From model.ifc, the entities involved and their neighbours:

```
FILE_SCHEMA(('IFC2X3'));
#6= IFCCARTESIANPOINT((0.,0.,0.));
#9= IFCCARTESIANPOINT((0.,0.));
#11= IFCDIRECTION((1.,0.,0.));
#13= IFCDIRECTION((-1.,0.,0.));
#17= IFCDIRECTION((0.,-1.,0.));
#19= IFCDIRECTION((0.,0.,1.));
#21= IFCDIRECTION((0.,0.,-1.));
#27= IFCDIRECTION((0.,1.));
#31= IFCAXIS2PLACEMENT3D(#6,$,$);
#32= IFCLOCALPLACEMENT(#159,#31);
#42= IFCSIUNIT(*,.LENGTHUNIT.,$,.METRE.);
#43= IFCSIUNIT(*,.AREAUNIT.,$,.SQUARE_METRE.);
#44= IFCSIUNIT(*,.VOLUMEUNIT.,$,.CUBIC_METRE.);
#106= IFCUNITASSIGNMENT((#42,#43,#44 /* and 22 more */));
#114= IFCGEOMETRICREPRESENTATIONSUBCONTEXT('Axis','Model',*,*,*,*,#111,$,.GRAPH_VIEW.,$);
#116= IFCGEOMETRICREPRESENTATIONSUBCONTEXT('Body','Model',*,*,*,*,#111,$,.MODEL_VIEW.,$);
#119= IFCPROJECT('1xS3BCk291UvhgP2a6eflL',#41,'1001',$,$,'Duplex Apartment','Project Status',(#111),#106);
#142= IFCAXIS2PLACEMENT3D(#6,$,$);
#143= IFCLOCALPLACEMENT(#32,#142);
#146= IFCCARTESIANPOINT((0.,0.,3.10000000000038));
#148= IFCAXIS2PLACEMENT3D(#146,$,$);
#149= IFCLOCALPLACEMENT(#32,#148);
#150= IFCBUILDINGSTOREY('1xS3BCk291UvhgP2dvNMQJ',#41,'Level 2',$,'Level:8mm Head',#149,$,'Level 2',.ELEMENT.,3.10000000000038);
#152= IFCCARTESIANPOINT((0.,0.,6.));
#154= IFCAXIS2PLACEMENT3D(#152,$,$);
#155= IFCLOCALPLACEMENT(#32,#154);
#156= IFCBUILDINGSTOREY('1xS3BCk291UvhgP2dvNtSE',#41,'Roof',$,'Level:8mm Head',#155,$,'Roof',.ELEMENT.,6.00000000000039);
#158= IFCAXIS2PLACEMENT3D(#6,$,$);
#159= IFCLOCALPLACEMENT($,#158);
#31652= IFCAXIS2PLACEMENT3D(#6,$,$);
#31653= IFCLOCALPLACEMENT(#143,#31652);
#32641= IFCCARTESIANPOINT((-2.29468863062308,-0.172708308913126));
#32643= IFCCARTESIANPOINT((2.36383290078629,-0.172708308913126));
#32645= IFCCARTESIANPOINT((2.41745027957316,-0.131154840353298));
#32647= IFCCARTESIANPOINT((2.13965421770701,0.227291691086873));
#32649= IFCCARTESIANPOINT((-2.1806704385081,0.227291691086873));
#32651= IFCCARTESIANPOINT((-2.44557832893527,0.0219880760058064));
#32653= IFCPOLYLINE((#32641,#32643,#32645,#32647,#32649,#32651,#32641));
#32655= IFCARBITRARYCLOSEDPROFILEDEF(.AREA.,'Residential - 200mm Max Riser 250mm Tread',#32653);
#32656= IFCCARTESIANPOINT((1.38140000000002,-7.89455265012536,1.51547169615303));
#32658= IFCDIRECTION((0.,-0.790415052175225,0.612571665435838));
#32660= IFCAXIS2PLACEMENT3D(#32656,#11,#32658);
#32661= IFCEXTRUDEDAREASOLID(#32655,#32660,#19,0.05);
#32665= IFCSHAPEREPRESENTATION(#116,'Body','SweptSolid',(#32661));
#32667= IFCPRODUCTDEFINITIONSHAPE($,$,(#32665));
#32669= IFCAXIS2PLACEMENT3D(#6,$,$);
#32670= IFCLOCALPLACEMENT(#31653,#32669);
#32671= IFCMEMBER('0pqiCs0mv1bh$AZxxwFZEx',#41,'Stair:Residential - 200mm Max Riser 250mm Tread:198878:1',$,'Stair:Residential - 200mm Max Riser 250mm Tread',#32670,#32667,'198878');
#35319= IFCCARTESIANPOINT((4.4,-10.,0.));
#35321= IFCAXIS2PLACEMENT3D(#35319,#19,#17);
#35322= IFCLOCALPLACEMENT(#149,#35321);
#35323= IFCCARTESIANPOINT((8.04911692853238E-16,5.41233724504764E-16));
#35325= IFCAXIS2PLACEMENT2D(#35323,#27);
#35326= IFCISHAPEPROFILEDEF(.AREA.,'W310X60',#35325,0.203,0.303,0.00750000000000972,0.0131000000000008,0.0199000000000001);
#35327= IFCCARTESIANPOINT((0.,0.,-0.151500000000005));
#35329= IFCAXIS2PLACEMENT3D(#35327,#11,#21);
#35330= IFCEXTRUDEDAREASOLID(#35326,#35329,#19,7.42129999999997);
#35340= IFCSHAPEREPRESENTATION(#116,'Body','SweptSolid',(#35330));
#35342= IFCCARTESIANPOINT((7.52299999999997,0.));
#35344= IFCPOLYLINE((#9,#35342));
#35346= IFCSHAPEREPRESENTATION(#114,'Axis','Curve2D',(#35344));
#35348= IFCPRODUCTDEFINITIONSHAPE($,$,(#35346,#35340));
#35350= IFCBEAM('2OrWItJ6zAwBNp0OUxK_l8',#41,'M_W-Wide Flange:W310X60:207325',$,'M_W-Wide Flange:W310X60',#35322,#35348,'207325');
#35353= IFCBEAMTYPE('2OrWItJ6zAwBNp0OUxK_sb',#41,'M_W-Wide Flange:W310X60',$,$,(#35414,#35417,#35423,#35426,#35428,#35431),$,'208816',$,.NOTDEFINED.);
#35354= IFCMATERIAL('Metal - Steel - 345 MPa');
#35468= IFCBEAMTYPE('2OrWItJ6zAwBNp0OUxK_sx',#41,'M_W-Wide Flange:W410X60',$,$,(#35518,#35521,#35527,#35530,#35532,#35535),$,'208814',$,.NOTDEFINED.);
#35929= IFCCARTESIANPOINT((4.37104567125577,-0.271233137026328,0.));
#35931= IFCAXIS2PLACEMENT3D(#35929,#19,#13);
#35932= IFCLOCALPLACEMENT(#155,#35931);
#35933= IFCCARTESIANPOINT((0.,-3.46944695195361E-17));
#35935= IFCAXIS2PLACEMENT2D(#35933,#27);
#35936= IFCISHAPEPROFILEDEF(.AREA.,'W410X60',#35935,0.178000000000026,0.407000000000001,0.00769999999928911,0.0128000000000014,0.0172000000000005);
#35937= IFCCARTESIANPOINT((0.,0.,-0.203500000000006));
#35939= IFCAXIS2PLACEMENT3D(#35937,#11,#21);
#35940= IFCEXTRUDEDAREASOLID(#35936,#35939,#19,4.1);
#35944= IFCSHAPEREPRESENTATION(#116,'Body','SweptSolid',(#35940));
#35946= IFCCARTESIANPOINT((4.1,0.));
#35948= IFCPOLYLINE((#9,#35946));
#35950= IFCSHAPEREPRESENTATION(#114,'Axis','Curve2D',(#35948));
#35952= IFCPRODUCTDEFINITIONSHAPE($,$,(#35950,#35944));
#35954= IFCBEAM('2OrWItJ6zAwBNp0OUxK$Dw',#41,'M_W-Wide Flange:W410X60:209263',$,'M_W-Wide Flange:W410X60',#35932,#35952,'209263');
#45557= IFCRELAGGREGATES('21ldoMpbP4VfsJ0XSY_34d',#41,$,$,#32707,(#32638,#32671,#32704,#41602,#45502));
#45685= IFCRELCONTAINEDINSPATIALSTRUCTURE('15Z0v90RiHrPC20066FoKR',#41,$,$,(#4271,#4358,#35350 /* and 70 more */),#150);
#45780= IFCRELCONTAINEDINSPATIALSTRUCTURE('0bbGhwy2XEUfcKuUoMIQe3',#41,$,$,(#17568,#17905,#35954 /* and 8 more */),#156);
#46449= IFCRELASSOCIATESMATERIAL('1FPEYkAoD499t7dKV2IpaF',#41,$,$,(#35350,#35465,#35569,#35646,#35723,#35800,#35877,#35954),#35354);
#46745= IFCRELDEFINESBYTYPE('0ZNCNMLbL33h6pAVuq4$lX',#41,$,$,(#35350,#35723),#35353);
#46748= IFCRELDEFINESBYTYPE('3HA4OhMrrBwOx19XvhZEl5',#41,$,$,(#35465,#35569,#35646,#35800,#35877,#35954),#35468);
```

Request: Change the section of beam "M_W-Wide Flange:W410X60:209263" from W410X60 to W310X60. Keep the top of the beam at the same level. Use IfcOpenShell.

```python
import ifcopenshell
import ifcopenshell.api.type
import ifcopenshell.util.element
import ifcopenshell.util.representation

model = ifcopenshell.open("model.ifc")

member = model.by_id(35954)
source = next(p for p in model.by_type("IfcIShapeProfileDef") if p.ProfileName == "W310X60")

body = ifcopenshell.util.representation.get_representation(member, "Model", "Body")
solid = body.Items[0]
old_profile = solid.SweptArea

# Copy the section's sizes but keep this member's own profile position.
profile = ifcopenshell.util.element.copy(model, source)
# Profiles are centred, so shift by half the change in depth to hold the top.
shift = (old_profile.OverallDepth - profile.OverallDepth) / 2
x, y = old_profile.Position.Location.Coordinates
up = (-1.0, 0.0)  # upwards, in the solid's own plane
location = model.createIfcCartesianPoint((x + up[0] * shift, y + up[1] * shift))
profile.Position = model.createIfcAxis2Placement2D(location, old_profile.Position.RefDirection)
solid.SweptArea = profile
if not model.get_total_inverses(old_profile):
    ifcopenshell.util.element.remove_deep2(model, old_profile)

new_type = model.by_guid("2OrWItJ6zAwBNp0OUxK_sb")
ifcopenshell.api.type.assign_type(
    model, related_objects=[member], relating_type=new_type, should_map_representations=False
)
member.Name = member.Name.replace("W410X60", "W310X60")
member.ObjectType = "M_W-Wide Flange:W310X60"

print(solid.SweptArea)

model.write("model_edited.ifc")
```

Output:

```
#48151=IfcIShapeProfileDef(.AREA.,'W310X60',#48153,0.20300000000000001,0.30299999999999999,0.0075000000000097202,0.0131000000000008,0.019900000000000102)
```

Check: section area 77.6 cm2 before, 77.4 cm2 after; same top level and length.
